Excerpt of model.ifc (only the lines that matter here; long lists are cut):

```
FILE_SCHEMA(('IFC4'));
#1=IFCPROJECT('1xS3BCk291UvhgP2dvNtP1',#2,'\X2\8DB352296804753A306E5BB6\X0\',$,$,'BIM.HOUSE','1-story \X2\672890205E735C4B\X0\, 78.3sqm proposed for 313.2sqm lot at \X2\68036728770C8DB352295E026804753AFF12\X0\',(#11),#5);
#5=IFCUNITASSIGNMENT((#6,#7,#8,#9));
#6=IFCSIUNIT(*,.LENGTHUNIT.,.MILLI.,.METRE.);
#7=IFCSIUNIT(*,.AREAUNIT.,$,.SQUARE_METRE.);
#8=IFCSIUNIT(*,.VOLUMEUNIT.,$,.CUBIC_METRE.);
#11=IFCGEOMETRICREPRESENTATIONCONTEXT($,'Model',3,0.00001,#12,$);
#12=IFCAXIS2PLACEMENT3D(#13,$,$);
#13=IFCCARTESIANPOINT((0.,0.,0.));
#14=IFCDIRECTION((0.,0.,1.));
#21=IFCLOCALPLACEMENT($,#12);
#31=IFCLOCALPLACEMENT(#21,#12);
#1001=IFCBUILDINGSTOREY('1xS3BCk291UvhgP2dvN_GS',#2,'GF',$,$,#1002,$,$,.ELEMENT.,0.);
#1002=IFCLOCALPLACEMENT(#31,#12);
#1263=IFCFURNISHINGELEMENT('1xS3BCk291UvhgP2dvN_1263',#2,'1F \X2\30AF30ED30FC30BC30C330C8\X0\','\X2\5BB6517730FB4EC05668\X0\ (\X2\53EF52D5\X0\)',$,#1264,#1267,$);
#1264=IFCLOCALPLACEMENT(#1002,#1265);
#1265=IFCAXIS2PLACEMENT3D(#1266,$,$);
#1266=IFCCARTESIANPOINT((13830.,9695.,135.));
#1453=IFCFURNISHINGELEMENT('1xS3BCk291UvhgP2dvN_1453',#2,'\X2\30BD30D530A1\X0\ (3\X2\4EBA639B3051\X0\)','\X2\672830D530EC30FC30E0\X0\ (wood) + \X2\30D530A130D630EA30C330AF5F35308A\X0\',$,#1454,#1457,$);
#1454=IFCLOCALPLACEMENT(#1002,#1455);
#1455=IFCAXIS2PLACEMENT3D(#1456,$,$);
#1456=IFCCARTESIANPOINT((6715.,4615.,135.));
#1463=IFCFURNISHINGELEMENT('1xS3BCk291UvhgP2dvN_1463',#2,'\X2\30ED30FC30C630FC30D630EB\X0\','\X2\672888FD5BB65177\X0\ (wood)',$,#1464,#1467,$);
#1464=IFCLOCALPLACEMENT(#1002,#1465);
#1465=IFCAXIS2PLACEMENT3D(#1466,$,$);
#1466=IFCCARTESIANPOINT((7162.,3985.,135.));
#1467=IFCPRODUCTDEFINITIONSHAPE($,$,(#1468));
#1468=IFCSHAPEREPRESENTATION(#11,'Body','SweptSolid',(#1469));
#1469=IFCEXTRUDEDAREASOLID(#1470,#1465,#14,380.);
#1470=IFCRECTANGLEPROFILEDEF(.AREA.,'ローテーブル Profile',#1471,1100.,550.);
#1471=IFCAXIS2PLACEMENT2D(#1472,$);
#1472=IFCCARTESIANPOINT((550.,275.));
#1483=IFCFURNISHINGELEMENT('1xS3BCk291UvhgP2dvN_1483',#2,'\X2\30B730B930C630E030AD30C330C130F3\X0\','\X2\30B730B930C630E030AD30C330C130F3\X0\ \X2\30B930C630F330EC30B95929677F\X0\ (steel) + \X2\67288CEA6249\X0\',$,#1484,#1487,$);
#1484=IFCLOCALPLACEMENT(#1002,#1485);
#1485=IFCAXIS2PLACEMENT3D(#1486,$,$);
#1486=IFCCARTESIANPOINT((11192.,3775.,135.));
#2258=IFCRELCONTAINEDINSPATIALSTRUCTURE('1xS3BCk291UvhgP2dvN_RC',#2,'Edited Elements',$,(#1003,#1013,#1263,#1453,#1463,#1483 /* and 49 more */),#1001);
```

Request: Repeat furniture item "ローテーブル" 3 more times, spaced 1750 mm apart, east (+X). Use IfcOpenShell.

```python
import numpy as np
import ifcopenshell
import ifcopenshell.api.geometry
import ifcopenshell.api.root
import ifcopenshell.util.element
import ifcopenshell.util.placement

model = ifcopenshell.open("model.ifc")


def reuse_history(source, copy):
    """copy_class also copies each property set's owner history, people and application; keep the originals."""
    for rel in copy.IsDefinedBy:
        if rel.is_a("IfcRelDefinesByProperties") and (history := rel.RelatingPropertyDefinition.OwnerHistory):
            rel.RelatingPropertyDefinition.OwnerHistory = source.OwnerHistory
            ifcopenshell.util.element.remove_deep2(model, history)


source = model.by_id(1463)
base = ifcopenshell.util.placement.get_local_placement(source.ObjectPlacement)
step = np.array([1.0, 0.0, 0.0]) * 1750.0

for i in range(1, 4):
    copy = ifcopenshell.api.root.copy_class(model, product=source)
    copy.Representation = ifcopenshell.util.element.copy_deep(
        model, source.Representation, exclude=["IfcGeometricRepresentationContext", "IfcRepresentationMap"]
    )
    reuse_history(source, copy)
    matrix = base.copy()
    matrix[:3, 3] += i * step
    print("added at", matrix[:3, 3].round(3) + 0.0)
    ifcopenshell.api.geometry.edit_object_placement(model, product=copy, matrix=matrix, is_si=False)

model.write("model_updated.ifc")
```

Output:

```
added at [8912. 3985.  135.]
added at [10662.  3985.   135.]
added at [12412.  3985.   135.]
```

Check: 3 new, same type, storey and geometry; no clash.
